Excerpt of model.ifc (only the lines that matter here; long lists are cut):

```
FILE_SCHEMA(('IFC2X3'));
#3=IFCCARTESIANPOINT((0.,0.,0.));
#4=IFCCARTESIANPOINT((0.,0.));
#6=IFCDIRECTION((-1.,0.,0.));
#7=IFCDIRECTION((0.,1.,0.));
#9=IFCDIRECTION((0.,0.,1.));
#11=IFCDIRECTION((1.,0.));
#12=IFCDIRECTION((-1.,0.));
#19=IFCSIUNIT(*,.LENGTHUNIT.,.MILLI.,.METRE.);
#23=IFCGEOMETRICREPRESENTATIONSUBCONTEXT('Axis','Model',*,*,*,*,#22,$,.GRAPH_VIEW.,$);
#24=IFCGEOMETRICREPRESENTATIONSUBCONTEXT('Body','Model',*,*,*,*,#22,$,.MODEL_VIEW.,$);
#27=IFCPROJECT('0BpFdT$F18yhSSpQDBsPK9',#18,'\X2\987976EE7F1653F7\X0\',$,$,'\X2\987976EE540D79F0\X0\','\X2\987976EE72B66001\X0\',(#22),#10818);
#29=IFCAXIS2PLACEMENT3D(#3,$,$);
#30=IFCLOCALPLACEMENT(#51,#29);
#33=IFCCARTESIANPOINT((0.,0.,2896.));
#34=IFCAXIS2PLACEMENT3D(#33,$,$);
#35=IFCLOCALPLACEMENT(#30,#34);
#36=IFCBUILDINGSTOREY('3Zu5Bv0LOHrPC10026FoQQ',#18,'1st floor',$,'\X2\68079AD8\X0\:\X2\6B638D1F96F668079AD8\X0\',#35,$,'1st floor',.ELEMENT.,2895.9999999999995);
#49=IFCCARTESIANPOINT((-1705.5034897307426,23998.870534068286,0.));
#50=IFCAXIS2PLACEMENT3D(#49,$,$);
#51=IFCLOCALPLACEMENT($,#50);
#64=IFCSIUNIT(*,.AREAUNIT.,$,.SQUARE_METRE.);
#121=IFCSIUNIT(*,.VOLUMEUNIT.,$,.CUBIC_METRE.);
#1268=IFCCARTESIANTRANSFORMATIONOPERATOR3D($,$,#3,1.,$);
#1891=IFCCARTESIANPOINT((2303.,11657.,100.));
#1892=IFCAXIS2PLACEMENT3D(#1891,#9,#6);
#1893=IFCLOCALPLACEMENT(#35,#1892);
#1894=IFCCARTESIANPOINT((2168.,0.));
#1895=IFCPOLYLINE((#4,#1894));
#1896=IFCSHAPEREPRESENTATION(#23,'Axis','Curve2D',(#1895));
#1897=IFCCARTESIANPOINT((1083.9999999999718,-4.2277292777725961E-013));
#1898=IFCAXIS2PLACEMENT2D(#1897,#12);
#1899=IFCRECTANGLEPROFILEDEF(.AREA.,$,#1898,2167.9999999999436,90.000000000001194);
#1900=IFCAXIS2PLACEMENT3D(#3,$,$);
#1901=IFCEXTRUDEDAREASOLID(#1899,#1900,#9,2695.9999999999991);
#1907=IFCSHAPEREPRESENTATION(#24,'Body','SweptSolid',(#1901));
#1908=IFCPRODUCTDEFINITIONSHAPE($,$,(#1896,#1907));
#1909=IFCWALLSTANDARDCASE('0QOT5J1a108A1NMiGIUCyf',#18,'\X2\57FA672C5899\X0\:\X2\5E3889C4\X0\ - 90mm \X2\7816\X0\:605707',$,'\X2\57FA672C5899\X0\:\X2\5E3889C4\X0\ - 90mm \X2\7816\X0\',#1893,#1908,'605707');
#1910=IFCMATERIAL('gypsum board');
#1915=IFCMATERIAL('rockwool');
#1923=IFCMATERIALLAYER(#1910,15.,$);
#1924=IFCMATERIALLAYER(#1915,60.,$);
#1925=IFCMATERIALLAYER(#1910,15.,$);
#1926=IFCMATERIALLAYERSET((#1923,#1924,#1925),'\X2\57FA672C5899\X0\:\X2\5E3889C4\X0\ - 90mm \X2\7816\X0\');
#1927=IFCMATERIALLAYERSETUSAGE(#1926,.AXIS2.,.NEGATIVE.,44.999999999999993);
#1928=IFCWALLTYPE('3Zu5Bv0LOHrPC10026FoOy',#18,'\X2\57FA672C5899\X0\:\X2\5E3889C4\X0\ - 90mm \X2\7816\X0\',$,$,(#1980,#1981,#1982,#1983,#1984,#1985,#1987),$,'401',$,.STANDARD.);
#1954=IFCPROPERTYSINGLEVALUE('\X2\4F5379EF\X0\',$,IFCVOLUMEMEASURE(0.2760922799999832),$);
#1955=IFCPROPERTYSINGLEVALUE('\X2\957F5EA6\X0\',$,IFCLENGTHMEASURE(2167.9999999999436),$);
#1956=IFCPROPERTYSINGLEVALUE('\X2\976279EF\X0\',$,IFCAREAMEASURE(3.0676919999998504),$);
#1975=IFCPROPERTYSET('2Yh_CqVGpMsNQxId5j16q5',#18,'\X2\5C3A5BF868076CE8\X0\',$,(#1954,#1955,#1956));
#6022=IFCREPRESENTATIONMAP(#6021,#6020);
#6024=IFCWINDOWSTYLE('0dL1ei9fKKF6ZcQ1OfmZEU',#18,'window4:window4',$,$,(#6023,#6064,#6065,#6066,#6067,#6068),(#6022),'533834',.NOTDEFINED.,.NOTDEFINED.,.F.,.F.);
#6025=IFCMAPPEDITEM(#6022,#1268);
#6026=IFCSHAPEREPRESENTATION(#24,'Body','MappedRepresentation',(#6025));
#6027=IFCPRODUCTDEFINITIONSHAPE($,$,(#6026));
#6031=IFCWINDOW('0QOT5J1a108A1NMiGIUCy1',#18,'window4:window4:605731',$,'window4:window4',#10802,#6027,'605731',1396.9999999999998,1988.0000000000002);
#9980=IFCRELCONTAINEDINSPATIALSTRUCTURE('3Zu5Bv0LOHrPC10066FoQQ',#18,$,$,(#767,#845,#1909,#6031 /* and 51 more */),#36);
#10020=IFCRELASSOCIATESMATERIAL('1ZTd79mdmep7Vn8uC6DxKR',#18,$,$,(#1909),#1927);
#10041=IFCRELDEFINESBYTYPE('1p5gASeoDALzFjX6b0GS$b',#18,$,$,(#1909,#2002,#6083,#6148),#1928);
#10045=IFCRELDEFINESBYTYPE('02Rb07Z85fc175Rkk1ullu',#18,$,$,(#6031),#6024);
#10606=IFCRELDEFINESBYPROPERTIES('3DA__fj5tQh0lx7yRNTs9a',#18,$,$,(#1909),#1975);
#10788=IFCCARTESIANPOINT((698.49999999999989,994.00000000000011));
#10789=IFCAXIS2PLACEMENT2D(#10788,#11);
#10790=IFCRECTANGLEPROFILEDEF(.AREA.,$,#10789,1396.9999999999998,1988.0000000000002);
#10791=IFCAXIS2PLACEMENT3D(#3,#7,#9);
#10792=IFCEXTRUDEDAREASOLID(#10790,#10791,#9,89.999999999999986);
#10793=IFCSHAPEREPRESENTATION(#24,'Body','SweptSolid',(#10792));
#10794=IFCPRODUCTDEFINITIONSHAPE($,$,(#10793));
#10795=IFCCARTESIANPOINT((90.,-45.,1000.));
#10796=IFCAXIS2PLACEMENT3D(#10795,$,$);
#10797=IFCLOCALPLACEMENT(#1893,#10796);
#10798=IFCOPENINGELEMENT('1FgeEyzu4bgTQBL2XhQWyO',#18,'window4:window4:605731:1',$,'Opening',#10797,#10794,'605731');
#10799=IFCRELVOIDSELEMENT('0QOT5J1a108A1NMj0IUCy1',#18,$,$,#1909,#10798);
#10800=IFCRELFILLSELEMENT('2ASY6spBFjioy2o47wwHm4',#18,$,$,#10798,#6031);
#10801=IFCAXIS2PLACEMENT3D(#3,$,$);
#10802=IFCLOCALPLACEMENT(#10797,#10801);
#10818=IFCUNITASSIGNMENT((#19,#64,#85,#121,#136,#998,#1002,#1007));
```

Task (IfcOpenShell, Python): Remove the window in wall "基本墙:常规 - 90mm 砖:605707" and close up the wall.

```python
import ifcopenshell
import ifcopenshell.api.feature
import ifcopenshell.api.pset
import ifcopenshell.api.root
import ifcopenshell.geom
import ifcopenshell.util.element
import ifcopenshell.util.shape
import ifcopenshell.util.unit

model = ifcopenshell.open("model.ifc")
area_scale = ifcopenshell.util.unit.calculate_unit_scale(model, "AREAUNIT")
volume_scale = ifcopenshell.util.unit.calculate_unit_scale(model, "VOLUMEUNIT")
settings = ifcopenshell.geom.settings()


def volume(element):
    """Net volume in cubic metres, openings subtracted."""
    shape = ifcopenshell.geom.create_shape(settings, element)
    return ifcopenshell.util.shape.get_volume(shape.geometry)


window = model.by_guid("0QOT5J1a108A1NMiGIUCy1")
opening = window.FillsVoids[0].RelatingOpeningElement
wall = opening.VoidsElements[0].RelatingBuildingElement
before = volume(wall)

ifcopenshell.api.root.remove_product(model, product=window)
ifcopenshell.api.feature.remove_feature(model, feature=opening)

after = volume(wall)
thickness = 0.09  # wall thickness in metres

# Update the wall's stored quantities.
pset = model.by_id(ifcopenshell.util.element.get_pset(wall, "尺寸标注", should_inherit=False)["id"])
ifcopenshell.api.pset.edit_pset(model, pset=pset, properties={
    "体积": model.create_entity("IfcVolumeMeasure", after / volume_scale),
    "面积": model.create_entity("IfcAreaMeasure", after / thickness / area_scale),
})

print(f"wall volume {before:.3f} -> {after:.3f} m3")

model.write("model_v2.ifc")
```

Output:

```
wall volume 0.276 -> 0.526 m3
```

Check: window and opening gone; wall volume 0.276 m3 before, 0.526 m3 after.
